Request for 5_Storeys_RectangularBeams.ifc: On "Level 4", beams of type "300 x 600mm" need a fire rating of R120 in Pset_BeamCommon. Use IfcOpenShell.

First a look at what the model holds.

```python
import ifcopenshell
import ifcopenshell.util.element

model = ifcopenshell.open("5_Storeys_RectangularBeams.ifc")
print(model.schema)
storey = next(s for s in model.by_type("IfcBuildingStorey") if s.Name == "Level 4")
beams = [e for e in ifcopenshell.util.element.get_decomposition(storey) if e.is_a("IfcBeam")]
seen = {}
for e in beams:
    element_type = ifcopenshell.util.element.get_type(e)
    key = (element_type.Name if element_type != e and element_type else None, ifcopenshell.util.element.get_pset(e, "Pset_BeamCommon", "FireRating"))
    seen[key] = seen.get(key, 0) + 1
for (name, value), count in sorted(seen.items(), key=str):
    print(count, "x", name, "|", value)
```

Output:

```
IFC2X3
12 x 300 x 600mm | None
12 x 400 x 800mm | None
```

```python
import ifcopenshell
import ifcopenshell.api.pset
import ifcopenshell.util.element

model = ifcopenshell.open("5_Storeys_RectangularBeams.ifc")

storey = next(s for s in model.by_type("IfcBuildingStorey") if s.Name == "Level 4")
beams = [e for e in ifcopenshell.util.element.get_decomposition(storey) if e.is_a("IfcBeam")]

count = 0
for e in beams:
    element_type = ifcopenshell.util.element.get_type(e)
    if element_type in (None, e) or element_type.Name != "300 x 600mm":
        continue
    # add_pset returns the element's existing set when there is one.
    pset = ifcopenshell.api.pset.add_pset(model, product=e, name="Pset_BeamCommon")
    ifcopenshell.api.pset.edit_pset(model, pset=pset, properties={"FireRating": "R120"})
    count += 1

print(count, "beams updated")

model.write("5_Storeys_RectangularBeams-out.ifc")
```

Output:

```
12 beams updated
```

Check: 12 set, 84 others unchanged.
